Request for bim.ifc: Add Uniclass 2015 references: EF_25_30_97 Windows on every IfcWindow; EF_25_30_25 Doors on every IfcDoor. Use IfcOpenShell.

First a look at what the model holds.

```python
import ifcopenshell

model = ifcopenshell.open("bim.ifc")
print(model.schema)
print("classifications:", [c.Name for c in model.by_type("IfcClassification")])
for ifc_class in ("IfcDoor", "IfcRoof", "IfcStair", "IfcWall", "IfcWindow"):
    print(ifc_class, len(model.by_type(ifc_class)))
```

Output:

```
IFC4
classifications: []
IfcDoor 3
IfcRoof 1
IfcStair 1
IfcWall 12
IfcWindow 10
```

```python
import ifcopenshell
import ifcopenshell.api.classification

model = ifcopenshell.open("bim.ifc")

system = ifcopenshell.api.classification.add_classification(model, classification="Uniclass 2015")

codes = {
    "IfcWindow": ("EF_25_30_97", "Windows"),
    "IfcDoor": ("EF_25_30_25", "Doors"),
}
for ifc_class, (code, name) in codes.items():
    products = model.by_type(ifc_class)
    ifcopenshell.api.classification.add_reference(
        model, products=products, classification=system, identification=code, name=name
    )
    print(code, len(products))

model.write("bim_v2.ifc")
```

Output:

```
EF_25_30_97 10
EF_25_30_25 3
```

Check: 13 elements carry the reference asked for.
